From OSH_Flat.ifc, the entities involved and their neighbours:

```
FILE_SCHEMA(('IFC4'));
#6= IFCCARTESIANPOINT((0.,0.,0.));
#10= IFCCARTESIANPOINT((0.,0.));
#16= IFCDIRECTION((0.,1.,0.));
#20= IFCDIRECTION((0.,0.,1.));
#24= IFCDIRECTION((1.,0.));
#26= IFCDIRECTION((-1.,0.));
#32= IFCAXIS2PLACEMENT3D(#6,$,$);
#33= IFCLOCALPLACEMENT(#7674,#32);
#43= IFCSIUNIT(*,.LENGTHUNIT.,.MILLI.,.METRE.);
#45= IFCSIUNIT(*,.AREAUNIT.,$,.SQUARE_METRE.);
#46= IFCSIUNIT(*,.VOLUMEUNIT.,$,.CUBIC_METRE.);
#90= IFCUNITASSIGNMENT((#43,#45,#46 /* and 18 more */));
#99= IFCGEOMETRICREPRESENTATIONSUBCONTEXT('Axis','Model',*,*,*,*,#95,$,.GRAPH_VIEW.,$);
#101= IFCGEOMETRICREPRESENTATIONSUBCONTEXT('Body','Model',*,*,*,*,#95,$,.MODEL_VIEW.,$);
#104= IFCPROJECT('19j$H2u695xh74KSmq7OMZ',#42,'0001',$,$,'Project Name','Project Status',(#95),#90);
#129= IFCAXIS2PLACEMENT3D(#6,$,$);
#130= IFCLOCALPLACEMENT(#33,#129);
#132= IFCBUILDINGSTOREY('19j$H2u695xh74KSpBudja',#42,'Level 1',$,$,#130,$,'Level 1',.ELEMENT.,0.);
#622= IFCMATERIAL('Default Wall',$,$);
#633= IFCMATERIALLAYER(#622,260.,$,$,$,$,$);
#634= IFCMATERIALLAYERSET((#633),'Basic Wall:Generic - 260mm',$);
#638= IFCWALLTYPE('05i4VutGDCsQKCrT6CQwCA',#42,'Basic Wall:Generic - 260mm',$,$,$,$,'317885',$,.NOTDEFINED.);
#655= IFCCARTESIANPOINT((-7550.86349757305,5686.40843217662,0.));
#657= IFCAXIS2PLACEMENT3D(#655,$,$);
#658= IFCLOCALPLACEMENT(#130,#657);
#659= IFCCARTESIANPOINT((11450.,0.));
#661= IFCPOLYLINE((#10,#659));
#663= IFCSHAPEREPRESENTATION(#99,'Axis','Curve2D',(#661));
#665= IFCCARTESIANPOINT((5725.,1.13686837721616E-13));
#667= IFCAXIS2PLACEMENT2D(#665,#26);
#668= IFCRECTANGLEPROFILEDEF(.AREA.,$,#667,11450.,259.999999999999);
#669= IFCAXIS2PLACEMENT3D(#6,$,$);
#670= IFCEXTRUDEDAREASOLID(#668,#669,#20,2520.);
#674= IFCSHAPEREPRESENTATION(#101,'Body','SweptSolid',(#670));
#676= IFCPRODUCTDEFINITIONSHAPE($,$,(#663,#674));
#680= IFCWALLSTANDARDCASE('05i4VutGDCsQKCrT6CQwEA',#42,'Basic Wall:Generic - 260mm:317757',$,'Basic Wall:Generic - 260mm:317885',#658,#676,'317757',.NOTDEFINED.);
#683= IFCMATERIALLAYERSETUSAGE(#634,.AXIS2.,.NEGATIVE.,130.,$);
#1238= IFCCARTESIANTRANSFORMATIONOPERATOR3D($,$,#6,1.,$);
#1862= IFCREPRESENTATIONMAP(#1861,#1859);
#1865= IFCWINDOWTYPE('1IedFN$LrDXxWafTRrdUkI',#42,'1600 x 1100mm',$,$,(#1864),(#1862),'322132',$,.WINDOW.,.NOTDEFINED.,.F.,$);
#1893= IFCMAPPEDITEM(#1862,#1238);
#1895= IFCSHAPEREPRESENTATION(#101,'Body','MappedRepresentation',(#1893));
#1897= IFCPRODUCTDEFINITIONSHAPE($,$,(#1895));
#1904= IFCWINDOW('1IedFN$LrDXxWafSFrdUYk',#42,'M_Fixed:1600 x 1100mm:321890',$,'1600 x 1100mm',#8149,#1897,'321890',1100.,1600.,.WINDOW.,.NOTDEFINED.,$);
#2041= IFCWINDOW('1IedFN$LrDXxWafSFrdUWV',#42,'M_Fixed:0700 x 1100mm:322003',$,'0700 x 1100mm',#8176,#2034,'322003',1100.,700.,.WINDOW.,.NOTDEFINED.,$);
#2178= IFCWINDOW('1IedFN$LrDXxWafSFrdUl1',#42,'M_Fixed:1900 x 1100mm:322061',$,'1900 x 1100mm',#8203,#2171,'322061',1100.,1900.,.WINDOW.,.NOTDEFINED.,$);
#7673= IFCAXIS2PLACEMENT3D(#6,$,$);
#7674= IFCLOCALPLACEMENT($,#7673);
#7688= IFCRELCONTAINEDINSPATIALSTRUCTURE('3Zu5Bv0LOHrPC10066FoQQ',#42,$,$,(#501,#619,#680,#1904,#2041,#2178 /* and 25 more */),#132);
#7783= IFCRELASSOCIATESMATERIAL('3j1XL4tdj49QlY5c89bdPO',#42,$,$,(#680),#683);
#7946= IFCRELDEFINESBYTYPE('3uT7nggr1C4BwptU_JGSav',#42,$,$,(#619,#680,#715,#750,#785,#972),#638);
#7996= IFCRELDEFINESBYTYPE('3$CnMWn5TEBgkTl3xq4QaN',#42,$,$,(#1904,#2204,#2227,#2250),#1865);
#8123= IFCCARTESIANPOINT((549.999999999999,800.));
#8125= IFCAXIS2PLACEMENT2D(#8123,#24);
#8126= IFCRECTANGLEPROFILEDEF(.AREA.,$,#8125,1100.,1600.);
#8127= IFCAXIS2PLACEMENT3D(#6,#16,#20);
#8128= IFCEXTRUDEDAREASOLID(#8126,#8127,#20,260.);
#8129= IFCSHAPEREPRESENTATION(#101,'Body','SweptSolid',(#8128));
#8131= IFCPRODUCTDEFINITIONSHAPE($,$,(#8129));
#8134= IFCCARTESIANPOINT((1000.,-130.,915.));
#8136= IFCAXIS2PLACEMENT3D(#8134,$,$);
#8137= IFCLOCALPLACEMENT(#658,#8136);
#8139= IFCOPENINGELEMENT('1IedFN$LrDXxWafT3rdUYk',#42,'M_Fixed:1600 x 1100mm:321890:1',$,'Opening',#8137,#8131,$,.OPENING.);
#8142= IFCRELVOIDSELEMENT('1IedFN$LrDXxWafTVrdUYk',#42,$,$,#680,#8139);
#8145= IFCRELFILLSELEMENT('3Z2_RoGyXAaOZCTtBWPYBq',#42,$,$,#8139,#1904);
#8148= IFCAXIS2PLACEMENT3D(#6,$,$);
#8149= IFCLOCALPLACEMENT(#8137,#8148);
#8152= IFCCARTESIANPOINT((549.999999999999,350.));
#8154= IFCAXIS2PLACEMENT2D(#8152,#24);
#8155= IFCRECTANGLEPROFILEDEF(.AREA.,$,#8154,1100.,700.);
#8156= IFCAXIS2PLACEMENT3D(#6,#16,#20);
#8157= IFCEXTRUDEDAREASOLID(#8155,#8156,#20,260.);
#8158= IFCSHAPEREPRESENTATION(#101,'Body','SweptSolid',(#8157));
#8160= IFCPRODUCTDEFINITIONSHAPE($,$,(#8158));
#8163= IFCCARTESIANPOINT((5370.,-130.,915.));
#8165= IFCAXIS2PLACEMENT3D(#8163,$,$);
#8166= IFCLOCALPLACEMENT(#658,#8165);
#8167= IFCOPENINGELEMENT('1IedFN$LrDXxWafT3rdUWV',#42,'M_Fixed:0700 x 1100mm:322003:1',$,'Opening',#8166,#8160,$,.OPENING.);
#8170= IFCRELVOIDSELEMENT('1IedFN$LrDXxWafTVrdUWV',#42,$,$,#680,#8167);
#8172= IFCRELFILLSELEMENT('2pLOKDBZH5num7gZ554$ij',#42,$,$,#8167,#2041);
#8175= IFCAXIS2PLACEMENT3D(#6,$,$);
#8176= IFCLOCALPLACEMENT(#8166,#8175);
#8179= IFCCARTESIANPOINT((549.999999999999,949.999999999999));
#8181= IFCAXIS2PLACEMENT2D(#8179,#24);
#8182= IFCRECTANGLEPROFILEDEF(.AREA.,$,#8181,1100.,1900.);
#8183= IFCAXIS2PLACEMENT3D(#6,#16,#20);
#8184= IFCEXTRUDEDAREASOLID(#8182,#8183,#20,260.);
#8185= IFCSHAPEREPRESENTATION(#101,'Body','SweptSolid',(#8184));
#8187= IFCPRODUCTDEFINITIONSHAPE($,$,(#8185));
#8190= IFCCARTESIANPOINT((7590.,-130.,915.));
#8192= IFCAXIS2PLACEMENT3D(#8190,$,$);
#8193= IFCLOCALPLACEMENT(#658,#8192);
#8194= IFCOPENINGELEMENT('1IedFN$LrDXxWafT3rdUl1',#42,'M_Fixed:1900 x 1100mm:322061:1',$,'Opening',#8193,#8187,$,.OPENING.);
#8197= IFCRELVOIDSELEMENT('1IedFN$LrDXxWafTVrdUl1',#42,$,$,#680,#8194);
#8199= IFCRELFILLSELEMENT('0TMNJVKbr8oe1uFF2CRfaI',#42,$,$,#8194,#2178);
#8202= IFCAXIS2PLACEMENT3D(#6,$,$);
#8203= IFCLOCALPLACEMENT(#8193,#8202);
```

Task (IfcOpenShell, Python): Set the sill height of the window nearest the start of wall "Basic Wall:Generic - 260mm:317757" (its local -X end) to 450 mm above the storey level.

```python
import numpy as np
import ifcopenshell
import ifcopenshell.api.geometry
import ifcopenshell.geom
import ifcopenshell.util.element
import ifcopenshell.util.placement
import ifcopenshell.util.shape
import ifcopenshell.util.unit

model = ifcopenshell.open("OSH_Flat.ifc")
unit_scale = ifcopenshell.util.unit.calculate_unit_scale(model)

window = model.by_guid("1IedFN$LrDXxWafSFrdUYk")
opening = window.FillsVoids[0].RelatingOpeningElement
storey = ifcopenshell.util.element.get_container(window, ifc_class="IfcBuildingStorey")
level = ifcopenshell.util.placement.get_local_placement(storey.ObjectPlacement)[2, 3]

# The opening's origin need not be at the sill, so measure its lowest point.
shape = ifcopenshell.geom.create_shape(ifcopenshell.geom.settings(), opening)
bottom = ifcopenshell.util.shape.get_shape_bottom_elevation(shape, shape.geometry) / unit_scale
dz = level + 0.45 / unit_scale - bottom

shift = np.array([0.0, 0.0, dz])
# The window is placed relative to its opening, so it follows when the opening moves.
matrix = ifcopenshell.util.placement.get_local_placement(opening.ObjectPlacement)
matrix[:3, 3] += shift
ifcopenshell.api.geometry.edit_object_placement(
    model, product=opening, matrix=matrix, is_si=False, should_transform_children=True
)

print(f"moved by {dz * unit_scale:+.3f} m")

model.write("OSH_Flat_updated.ifc")
```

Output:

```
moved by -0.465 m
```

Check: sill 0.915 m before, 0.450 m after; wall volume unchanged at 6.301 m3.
